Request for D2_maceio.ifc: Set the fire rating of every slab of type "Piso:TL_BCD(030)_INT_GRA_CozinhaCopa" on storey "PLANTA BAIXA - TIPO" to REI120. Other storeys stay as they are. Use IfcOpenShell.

First a look at what the model holds.

```python
import ifcopenshell
import ifcopenshell.util.element

model = ifcopenshell.open("D2_maceio.ifc")
print(model.schema)
storey = next(s for s in model.by_type("IfcBuildingStorey") if s.Name == "PLANTA BAIXA - TIPO")
slabs = [e for e in ifcopenshell.util.element.get_decomposition(storey) if e.is_a("IfcSlab")]
seen = {}
for e in slabs:
    element_type = ifcopenshell.util.element.get_type(e)
    key = (element_type.Name if element_type != e and element_type else None, ifcopenshell.util.element.get_pset(e, "Pset_SlabCommon", "FireRating"))
    seen[key] = seen.get(key, 0) + 1
for (name, value), count in sorted(seen.items(), key=str):
    print(count, "x", name, "|", value)
```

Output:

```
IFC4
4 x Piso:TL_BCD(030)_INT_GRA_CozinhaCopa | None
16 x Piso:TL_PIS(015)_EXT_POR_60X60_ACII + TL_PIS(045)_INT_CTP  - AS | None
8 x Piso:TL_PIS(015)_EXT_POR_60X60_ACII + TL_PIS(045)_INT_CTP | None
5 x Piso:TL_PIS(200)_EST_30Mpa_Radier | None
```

```python
import ifcopenshell
import ifcopenshell.api.pset
import ifcopenshell.util.element

model = ifcopenshell.open("D2_maceio.ifc")

storey = next(s for s in model.by_type("IfcBuildingStorey") if s.Name == "PLANTA BAIXA - TIPO")
slabs = [e for e in ifcopenshell.util.element.get_decomposition(storey) if e.is_a("IfcSlab")]

count = 0
for e in slabs:
    element_type = ifcopenshell.util.element.get_type(e)
    if element_type in (None, e) or element_type.Name != "Piso:TL_BCD(030)_INT_GRA_CozinhaCopa":
        continue
    # add_pset returns the element's existing set when there is one.
    pset = ifcopenshell.api.pset.add_pset(model, product=e, name="Pset_SlabCommon")
    ifcopenshell.api.pset.edit_pset(model, pset=pset, properties={"FireRating": "REI120"})
    count += 1

print(count, "slabs updated")

model.write("D2_maceio_rev.ifc")
```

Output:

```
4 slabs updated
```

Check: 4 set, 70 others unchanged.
